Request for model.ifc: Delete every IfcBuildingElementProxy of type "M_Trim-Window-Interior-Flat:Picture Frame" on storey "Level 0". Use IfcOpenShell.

First a look at what the model holds.

```python
import ifcopenshell
import ifcopenshell.util.element

model = ifcopenshell.open("model.ifc")
print(model.schema)
storey = next(s for s in model.by_type("IfcBuildingStorey") if s.Name == "Level 0")
proxies = [e for e in ifcopenshell.util.element.get_decomposition(storey) if e.is_a("IfcBuildingElementProxy")]
seen = {}
for e in proxies:
    element_type = ifcopenshell.util.element.get_type(e)
    name = element_type.Name if element_type not in (None, e) else None
    seen[name] = seen.get(name, 0) + 1
for name, count in sorted(seen.items(), key=str):
    print(count, "x", name)
```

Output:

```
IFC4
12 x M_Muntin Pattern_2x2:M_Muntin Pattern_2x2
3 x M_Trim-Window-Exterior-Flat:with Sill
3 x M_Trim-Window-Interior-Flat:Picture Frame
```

```python
import ifcopenshell
import ifcopenshell.api.root
import ifcopenshell.util.element

model = ifcopenshell.open("model.ifc")

storey = next(s for s in model.by_type("IfcBuildingStorey") if s.Name == "Level 0")
proxies = [e for e in ifcopenshell.util.element.get_decomposition(storey) if e.is_a("IfcBuildingElementProxy")]
targets = [e for e in proxies if (t := ifcopenshell.util.element.get_type(e)) not in (None, e) and t.Name == "M_Trim-Window-Interior-Flat:Picture Frame"]

for e in targets:
    ifcopenshell.api.root.remove_product(model, product=e)
print(len(targets), "removed")

model.write("model_edited.ifc")
```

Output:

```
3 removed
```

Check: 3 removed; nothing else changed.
